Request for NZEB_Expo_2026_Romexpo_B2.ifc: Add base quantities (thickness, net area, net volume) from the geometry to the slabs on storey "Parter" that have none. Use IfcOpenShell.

First a look at what the model holds.

```python
import ifcopenshell
import ifcopenshell.util.element
import ifcopenshell.util.unit

model = ifcopenshell.open("NZEB_Expo_2026_Romexpo_B2.ifc")
print(model.schema)
for unit_type in ("LENGTHUNIT", "AREAUNIT", "VOLUMEUNIT"):
    print(unit_type, ifcopenshell.util.unit.calculate_unit_scale(model, unit_type))
storey = next(s for s in model.by_type("IfcBuildingStorey") if s.Name == "Parter")
slabs = [e for e in ifcopenshell.util.element.get_decomposition(storey) if e.is_a("IfcSlab")]
for e in sorted(slabs, key=lambda e: e.id()):
    print(e.id(), e.is_a(), e.Name, list(ifcopenshell.util.element.get_psets(e, qtos_only=True)), sep=" | ")
```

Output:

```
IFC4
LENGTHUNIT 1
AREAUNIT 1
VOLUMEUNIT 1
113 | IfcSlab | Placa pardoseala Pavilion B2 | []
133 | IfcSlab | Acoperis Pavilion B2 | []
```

```python
import ifcopenshell
import ifcopenshell.api.pset
import ifcopenshell.geom
import ifcopenshell.util.element
import ifcopenshell.util.shape
import ifcopenshell.util.unit

model = ifcopenshell.open("NZEB_Expo_2026_Romexpo_B2.ifc")
unit_scale = ifcopenshell.util.unit.calculate_unit_scale(model)
area_scale = ifcopenshell.util.unit.calculate_unit_scale(model, "AREAUNIT")
volume_scale = ifcopenshell.util.unit.calculate_unit_scale(model, "VOLUMEUNIT")
settings = ifcopenshell.geom.settings()

storey = next(s for s in model.by_type("IfcBuildingStorey") if s.Name == "Parter")
slabs = [e for e in ifcopenshell.util.element.get_decomposition(storey) if e.is_a("IfcSlab")]

for e in sorted(slabs, key=lambda e: e.id()):
    if ifcopenshell.util.element.get_psets(e, qtos_only=True, should_inherit=False):
        continue
    # Geometry comes back in metres, in the element's own axes.
    shape = ifcopenshell.geom.create_shape(settings, e)
    values = {
        "Width": ifcopenshell.util.shape.get_z(shape.geometry) / unit_scale,
        "NetArea": ifcopenshell.util.shape.get_footprint_area(shape.geometry) / area_scale,
        "NetVolume": ifcopenshell.util.shape.get_volume(shape.geometry) / volume_scale,
    }
    qto = ifcopenshell.api.pset.add_qto(model, product=e, name="Qto_SlabBaseQuantities")
    ifcopenshell.api.pset.edit_qto(model, qto=qto, properties=values)
    print(e.id(), {k: round(v, 3) for k, v in values.items()})

model.write("NZEB_Expo_2026_Romexpo_B2_v2.ifc")
```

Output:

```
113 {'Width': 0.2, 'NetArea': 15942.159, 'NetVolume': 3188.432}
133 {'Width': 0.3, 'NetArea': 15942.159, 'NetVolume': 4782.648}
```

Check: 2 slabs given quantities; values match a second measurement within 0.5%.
